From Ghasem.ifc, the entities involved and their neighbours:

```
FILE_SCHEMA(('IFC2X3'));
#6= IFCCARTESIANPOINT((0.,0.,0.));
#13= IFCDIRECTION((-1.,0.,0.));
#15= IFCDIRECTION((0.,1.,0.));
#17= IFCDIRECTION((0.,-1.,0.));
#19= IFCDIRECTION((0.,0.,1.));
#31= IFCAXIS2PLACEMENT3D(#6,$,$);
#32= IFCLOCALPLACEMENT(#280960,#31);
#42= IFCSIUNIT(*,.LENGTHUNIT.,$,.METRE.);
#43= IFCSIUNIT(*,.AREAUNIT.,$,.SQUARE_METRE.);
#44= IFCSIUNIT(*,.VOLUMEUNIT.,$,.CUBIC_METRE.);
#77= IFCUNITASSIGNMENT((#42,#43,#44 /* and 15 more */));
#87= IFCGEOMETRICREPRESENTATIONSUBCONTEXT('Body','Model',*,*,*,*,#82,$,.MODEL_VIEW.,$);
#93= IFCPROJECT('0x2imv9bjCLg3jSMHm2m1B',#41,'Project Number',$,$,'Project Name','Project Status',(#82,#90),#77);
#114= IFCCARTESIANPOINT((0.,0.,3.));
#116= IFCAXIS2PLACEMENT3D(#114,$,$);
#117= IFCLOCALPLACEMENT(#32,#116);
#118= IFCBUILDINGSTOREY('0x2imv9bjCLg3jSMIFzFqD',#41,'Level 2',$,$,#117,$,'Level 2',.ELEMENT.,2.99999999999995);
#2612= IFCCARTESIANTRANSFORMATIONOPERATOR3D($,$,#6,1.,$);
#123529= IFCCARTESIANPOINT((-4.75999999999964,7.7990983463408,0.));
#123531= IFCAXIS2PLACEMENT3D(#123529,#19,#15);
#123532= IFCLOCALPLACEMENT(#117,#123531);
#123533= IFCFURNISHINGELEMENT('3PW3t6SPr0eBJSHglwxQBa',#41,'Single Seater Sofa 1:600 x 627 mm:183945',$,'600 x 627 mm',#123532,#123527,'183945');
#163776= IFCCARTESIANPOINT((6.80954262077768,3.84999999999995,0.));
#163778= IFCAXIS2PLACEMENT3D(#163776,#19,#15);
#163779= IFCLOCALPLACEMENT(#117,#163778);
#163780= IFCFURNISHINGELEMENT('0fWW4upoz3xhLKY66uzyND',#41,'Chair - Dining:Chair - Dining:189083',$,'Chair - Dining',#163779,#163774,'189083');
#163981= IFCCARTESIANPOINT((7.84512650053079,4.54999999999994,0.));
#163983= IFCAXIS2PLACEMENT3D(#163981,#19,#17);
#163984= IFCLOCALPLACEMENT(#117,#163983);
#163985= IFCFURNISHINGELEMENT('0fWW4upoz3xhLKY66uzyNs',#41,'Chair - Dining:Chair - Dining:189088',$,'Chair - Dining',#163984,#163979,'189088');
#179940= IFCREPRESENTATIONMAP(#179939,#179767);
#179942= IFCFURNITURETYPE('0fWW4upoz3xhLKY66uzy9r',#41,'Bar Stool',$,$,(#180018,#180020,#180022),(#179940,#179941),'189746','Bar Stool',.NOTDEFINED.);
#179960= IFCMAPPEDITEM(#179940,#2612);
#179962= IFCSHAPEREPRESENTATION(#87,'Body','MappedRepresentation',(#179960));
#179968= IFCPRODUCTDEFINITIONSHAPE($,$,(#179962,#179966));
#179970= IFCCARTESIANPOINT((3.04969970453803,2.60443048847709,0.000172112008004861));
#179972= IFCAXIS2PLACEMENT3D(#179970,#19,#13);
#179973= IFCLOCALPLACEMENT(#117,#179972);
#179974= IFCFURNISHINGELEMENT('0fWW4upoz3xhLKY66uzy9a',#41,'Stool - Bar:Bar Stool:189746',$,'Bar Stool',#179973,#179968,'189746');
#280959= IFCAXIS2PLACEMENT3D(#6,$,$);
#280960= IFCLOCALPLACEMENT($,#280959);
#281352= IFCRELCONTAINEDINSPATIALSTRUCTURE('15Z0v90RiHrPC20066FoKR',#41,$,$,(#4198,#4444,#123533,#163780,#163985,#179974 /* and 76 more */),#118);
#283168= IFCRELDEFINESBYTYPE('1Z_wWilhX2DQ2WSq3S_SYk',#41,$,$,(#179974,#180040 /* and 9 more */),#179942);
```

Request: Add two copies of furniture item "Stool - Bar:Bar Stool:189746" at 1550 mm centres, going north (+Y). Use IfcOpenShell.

```python
import numpy as np
import ifcopenshell
import ifcopenshell.api.geometry
import ifcopenshell.api.root
import ifcopenshell.util.element
import ifcopenshell.util.placement
import ifcopenshell.util.unit

model = ifcopenshell.open("Ghasem.ifc")
unit_scale = ifcopenshell.util.unit.calculate_unit_scale(model)


def reuse_history(source, copy):
    """copy_class also copies each property set's owner history, people and application; keep the originals."""
    for rel in copy.IsDefinedBy:
        if rel.is_a("IfcRelDefinesByProperties") and (history := rel.RelatingPropertyDefinition.OwnerHistory):
            rel.RelatingPropertyDefinition.OwnerHistory = source.OwnerHistory
            ifcopenshell.util.element.remove_deep2(model, history)


source = model.by_id(179974)
base = ifcopenshell.util.placement.get_local_placement(source.ObjectPlacement)
step = np.array([0.0, 1.0, 0.0]) * 1.55 / unit_scale

for i in range(1, 3):
    copy = ifcopenshell.api.root.copy_class(model, product=source)
    copy.Representation = ifcopenshell.util.element.copy_deep(
        model, source.Representation, exclude=["IfcGeometricRepresentationContext", "IfcRepresentationMap"]
    )
    copy.Name = "Stool - Bar:Bar Stool"
    copy.Tag = None
    reuse_history(source, copy)
    matrix = base.copy()
    matrix[:3, 3] += i * step
    print("added at", matrix[:3, 3].round(3) + 0.0)
    ifcopenshell.api.geometry.edit_object_placement(model, product=copy, matrix=matrix, is_si=False)

model.write("Ghasem_updated.ifc")
```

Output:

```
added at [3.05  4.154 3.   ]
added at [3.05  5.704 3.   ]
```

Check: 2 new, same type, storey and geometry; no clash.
